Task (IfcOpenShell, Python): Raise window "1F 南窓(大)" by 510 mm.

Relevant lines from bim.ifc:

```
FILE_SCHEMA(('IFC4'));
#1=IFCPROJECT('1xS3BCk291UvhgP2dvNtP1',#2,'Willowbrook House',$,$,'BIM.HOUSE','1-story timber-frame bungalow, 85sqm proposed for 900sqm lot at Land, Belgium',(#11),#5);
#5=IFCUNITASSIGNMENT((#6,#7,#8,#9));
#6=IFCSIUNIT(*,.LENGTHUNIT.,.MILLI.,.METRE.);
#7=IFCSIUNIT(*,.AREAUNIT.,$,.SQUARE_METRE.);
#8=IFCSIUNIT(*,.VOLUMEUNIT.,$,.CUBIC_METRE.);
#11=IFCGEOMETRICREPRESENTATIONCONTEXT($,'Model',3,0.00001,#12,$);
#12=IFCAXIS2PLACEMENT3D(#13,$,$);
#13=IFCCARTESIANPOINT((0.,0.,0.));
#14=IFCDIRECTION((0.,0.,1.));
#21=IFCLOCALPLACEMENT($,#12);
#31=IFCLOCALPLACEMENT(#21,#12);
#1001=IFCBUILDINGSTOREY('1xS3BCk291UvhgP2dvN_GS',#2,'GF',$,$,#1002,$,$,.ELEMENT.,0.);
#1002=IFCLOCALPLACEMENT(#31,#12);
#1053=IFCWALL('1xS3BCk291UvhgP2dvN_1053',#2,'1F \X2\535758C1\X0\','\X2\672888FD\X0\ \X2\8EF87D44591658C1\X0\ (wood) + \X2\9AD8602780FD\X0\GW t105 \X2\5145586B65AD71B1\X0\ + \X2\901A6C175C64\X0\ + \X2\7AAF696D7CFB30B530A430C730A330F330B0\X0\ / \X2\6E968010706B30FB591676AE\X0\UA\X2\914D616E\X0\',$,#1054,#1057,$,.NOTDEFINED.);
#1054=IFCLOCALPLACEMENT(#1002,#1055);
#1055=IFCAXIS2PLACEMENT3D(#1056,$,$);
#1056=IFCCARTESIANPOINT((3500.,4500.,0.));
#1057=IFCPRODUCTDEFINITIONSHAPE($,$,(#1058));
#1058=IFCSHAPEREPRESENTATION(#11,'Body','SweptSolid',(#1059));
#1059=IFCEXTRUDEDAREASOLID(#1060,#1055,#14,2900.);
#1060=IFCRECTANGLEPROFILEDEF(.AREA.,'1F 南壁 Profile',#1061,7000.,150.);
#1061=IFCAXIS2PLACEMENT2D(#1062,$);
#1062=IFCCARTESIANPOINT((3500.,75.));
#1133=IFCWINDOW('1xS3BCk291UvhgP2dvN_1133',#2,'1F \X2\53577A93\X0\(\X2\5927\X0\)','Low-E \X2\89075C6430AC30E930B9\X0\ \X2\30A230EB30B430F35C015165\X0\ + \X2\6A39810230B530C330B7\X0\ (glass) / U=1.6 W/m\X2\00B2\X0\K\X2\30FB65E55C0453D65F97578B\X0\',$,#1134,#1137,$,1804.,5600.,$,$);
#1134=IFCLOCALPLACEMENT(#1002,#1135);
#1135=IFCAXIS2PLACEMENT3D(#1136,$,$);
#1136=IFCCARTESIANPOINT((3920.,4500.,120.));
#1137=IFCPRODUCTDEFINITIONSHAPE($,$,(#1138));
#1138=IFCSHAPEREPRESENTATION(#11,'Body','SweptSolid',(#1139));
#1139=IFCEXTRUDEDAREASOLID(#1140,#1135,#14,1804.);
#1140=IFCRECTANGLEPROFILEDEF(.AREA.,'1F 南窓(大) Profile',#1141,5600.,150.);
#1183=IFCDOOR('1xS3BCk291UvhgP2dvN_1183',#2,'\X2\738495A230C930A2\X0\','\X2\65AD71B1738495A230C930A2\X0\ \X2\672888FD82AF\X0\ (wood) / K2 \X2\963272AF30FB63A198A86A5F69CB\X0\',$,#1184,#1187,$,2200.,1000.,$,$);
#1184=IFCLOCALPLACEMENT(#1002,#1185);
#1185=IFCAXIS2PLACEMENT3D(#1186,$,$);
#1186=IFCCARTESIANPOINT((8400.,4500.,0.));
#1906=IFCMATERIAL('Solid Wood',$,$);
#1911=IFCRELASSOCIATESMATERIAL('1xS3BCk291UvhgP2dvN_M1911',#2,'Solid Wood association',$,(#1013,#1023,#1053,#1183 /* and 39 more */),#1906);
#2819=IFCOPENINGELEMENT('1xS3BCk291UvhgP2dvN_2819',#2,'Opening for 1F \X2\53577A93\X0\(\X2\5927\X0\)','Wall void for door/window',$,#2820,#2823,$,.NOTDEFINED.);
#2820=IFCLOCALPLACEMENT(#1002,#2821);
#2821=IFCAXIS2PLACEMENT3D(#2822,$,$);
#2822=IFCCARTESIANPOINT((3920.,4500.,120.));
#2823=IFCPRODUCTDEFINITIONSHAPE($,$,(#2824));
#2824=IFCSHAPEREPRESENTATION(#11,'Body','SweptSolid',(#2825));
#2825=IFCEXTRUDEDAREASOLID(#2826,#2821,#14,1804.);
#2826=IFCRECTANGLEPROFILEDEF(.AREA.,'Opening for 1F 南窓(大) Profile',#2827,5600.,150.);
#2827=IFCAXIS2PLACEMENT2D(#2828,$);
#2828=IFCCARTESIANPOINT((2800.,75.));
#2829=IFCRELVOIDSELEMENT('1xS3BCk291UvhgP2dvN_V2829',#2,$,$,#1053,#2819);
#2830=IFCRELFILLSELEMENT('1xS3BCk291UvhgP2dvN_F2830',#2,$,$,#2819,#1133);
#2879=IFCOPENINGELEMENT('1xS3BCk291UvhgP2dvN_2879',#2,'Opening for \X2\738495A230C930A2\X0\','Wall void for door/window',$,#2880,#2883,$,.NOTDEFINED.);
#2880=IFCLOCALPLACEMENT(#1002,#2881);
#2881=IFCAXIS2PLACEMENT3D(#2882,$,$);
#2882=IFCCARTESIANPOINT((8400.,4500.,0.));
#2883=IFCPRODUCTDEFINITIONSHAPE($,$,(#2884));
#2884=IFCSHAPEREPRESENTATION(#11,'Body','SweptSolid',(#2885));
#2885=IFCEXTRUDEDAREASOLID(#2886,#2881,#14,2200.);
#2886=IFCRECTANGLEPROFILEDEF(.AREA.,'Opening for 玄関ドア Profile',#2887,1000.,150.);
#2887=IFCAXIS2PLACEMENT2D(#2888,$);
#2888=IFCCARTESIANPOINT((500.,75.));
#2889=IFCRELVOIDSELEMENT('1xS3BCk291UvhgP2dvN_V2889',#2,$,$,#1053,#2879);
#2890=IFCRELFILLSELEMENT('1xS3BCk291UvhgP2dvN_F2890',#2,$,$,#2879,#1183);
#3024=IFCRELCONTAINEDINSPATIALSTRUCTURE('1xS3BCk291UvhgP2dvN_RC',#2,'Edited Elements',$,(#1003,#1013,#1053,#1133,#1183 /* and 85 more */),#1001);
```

```python
import numpy as np
import ifcopenshell
import ifcopenshell.api.geometry
import ifcopenshell.util.placement
import ifcopenshell.util.unit

model = ifcopenshell.open("bim.ifc")
unit_scale = ifcopenshell.util.unit.calculate_unit_scale(model)

window = model.by_guid("1xS3BCk291UvhgP2dvN_1133")
opening = window.FillsVoids[0].RelatingOpeningElement
dz = 0.51 / unit_scale

shift = np.array([0.0, 0.0, dz])
# The window is not placed relative to its opening, so move both.
for product in (opening, window):
    matrix = ifcopenshell.util.placement.get_local_placement(product.ObjectPlacement)
    matrix[:3, 3] += shift
    ifcopenshell.api.geometry.edit_object_placement(model, product=product, matrix=matrix, is_si=False)

print(f"moved by {dz * unit_scale:+.3f} m")

model.write("bim_updated.ifc")
```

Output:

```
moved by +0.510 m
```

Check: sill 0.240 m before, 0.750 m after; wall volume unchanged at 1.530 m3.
